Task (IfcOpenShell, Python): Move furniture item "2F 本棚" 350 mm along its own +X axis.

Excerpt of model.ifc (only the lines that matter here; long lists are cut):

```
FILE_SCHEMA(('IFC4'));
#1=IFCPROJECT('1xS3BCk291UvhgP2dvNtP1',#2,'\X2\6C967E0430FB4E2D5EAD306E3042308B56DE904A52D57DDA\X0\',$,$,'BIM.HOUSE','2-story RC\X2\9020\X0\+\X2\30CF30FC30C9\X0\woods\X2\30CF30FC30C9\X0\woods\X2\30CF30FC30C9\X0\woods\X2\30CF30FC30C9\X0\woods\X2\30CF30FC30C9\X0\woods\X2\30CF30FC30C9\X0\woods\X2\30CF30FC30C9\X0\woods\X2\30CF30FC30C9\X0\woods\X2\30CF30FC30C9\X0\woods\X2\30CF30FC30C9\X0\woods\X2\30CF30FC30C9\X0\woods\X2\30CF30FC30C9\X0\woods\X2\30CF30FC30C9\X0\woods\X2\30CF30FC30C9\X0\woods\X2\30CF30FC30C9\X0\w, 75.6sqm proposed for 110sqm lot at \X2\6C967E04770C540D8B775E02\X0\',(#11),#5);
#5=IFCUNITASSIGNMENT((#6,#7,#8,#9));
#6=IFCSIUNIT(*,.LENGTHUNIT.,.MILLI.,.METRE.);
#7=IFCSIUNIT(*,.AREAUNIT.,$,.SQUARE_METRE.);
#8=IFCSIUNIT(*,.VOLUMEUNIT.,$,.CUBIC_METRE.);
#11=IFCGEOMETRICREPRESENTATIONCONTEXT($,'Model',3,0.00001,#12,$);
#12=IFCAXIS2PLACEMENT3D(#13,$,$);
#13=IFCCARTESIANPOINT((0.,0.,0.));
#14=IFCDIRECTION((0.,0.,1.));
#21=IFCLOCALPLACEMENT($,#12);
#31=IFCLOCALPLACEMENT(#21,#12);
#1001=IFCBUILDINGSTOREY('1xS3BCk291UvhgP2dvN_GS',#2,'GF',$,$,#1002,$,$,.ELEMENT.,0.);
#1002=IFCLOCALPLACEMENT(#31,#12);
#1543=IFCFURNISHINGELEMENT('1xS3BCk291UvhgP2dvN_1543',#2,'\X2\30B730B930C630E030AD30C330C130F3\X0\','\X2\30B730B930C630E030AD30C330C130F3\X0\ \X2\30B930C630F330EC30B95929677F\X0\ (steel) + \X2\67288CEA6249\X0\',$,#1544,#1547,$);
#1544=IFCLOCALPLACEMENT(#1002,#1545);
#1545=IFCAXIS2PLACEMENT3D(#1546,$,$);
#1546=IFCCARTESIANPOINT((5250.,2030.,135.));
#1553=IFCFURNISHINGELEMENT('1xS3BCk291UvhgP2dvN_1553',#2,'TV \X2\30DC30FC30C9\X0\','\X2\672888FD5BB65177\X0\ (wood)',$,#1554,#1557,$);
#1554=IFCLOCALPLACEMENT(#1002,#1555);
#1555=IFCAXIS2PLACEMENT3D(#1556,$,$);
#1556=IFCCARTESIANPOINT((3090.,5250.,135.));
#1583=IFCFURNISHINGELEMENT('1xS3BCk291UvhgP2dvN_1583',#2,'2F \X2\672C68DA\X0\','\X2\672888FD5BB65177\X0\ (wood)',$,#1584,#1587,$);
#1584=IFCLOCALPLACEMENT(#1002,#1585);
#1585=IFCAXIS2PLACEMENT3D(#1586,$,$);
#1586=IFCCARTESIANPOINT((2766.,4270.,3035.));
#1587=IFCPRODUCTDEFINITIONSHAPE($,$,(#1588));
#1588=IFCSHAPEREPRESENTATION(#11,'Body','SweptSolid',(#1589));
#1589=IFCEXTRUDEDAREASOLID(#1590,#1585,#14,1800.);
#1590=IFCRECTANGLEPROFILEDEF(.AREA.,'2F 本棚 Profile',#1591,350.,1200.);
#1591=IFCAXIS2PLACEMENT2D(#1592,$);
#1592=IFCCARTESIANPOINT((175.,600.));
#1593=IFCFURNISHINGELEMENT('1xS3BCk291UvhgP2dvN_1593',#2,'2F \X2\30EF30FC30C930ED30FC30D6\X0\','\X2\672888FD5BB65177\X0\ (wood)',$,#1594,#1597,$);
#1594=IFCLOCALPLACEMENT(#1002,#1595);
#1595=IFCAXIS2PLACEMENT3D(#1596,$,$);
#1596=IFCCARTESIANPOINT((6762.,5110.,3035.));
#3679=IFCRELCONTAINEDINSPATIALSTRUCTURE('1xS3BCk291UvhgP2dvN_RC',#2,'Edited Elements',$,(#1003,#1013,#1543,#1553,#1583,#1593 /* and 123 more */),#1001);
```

```python
import ifcopenshell
import ifcopenshell.api.geometry
import ifcopenshell.util.placement
import ifcopenshell.util.unit

model = ifcopenshell.open("model.ifc")
unit_scale = ifcopenshell.util.unit.calculate_unit_scale(model)

item = model.by_guid("1xS3BCk291UvhgP2dvN_1583")
matrix = ifcopenshell.util.placement.get_local_placement(item.ObjectPlacement)
matrix[:3, 3] += matrix[:3, 0] * 0.35 / unit_scale
ifcopenshell.api.geometry.edit_object_placement(model, product=item, matrix=matrix, is_si=False)

print(ifcopenshell.util.placement.get_local_placement(item.ObjectPlacement).round(3) + 0.0)

model.write("model-out.ifc")
```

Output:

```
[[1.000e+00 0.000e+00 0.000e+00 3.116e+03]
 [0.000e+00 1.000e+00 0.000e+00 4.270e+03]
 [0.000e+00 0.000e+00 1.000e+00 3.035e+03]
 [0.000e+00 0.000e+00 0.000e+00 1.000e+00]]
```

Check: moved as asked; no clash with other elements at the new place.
